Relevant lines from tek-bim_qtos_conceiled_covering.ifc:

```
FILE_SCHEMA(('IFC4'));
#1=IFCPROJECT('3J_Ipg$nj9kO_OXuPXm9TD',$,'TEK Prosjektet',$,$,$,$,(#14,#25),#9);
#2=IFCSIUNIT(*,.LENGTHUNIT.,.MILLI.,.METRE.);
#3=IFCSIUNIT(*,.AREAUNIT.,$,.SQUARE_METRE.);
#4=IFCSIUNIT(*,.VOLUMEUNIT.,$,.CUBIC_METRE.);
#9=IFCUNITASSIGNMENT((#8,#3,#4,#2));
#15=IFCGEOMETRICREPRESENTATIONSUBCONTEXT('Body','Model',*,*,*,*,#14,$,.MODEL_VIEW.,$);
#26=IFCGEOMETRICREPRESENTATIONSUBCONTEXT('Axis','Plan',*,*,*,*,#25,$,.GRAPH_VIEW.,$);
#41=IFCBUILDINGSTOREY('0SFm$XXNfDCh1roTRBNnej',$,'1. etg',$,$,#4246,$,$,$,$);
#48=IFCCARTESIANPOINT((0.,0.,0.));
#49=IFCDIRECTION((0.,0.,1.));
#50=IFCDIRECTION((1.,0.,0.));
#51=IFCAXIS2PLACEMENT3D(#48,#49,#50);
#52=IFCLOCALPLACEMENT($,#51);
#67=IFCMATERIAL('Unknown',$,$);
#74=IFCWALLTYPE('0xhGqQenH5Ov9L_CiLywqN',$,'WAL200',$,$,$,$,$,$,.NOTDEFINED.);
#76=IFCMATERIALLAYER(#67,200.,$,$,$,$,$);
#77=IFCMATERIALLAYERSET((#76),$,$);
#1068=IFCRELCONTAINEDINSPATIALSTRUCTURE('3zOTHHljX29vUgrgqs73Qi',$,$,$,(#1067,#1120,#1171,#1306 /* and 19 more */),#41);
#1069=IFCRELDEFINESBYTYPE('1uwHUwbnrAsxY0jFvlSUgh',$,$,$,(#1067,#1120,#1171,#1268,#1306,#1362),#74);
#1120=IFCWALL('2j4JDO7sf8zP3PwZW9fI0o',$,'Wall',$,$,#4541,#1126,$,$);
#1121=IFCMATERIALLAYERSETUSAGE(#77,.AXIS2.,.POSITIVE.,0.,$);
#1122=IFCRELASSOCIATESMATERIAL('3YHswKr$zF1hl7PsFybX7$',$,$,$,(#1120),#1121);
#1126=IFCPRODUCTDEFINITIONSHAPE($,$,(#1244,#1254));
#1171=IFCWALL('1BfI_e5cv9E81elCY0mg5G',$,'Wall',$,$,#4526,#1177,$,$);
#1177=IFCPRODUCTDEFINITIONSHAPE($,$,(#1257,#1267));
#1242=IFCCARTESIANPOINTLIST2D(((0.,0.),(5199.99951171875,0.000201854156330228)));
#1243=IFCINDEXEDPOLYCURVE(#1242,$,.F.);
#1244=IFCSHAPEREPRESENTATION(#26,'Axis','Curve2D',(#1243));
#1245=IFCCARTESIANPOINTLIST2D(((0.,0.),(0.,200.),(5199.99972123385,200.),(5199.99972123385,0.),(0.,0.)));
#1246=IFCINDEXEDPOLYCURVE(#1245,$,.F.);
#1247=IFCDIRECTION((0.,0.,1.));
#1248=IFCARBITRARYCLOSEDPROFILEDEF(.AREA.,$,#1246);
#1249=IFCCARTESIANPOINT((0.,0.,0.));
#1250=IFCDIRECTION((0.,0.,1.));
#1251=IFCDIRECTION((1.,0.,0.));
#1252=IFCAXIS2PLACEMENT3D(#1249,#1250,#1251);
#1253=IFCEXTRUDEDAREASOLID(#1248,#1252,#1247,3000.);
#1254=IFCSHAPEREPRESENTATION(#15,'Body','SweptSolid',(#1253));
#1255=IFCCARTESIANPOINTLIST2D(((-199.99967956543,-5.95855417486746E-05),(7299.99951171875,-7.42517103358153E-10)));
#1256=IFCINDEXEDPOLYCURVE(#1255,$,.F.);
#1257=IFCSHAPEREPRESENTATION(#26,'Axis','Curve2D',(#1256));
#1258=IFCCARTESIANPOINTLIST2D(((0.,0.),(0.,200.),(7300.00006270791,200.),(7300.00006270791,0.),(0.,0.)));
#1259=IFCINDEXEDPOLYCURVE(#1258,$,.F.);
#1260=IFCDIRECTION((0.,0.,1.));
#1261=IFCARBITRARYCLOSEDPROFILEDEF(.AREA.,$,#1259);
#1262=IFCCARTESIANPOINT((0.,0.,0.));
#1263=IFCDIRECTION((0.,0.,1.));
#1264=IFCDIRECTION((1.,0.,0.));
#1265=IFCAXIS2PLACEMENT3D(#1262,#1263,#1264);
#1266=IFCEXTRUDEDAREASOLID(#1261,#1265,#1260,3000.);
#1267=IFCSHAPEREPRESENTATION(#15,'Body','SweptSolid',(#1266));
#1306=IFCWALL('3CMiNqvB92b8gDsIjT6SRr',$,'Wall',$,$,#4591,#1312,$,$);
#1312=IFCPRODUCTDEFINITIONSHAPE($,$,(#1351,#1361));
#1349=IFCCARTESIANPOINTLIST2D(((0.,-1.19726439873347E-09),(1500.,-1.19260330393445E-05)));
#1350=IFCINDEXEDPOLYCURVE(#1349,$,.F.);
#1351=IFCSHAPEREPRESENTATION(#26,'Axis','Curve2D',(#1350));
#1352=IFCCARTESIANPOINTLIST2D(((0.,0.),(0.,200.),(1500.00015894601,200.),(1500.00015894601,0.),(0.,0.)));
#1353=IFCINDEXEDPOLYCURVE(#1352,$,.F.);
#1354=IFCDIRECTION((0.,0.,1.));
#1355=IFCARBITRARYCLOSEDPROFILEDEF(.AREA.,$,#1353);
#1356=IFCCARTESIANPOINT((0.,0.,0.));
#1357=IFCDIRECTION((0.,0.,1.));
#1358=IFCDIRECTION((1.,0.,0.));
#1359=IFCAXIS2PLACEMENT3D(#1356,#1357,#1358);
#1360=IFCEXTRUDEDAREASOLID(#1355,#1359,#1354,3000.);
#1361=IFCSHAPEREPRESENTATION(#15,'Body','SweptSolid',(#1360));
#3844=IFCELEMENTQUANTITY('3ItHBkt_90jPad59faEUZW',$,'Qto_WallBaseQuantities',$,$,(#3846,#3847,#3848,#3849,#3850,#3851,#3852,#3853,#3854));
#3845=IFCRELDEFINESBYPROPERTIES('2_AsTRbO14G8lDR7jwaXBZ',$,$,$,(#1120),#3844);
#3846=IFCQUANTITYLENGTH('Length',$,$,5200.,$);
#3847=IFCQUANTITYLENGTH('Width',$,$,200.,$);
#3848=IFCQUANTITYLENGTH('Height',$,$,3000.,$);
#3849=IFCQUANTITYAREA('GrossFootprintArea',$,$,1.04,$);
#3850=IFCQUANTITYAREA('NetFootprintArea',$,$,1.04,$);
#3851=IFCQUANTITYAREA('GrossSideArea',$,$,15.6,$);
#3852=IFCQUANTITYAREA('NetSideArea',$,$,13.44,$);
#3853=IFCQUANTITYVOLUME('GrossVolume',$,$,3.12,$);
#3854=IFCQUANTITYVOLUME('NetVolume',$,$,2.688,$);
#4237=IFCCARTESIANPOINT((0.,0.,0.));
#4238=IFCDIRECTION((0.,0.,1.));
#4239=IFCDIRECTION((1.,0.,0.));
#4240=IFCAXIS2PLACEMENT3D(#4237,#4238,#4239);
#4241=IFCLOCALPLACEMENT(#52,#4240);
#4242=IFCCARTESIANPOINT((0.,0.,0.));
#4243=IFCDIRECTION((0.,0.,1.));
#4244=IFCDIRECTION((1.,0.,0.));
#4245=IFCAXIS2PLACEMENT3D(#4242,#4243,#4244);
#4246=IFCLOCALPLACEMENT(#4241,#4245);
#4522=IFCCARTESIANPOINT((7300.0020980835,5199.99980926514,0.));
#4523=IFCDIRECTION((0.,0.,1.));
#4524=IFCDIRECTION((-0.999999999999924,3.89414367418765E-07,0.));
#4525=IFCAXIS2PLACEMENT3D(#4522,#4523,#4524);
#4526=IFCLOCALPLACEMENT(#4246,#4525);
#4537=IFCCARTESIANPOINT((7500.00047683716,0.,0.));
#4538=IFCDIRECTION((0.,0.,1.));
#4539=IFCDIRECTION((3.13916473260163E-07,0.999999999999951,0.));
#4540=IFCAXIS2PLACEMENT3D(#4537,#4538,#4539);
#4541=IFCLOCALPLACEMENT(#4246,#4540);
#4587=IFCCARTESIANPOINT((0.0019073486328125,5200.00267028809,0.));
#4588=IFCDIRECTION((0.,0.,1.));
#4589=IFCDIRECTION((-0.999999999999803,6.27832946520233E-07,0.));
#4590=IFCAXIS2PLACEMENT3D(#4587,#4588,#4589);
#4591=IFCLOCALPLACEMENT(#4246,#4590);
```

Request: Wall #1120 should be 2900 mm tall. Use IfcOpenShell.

```python
import ifcopenshell
import ifcopenshell.api.pset
import ifcopenshell.geom
import ifcopenshell.util.element
import ifcopenshell.util.representation
import ifcopenshell.util.shape
import ifcopenshell.util.unit

model = ifcopenshell.open("tek-bim_qtos_conceiled_covering.ifc")
unit_scale = ifcopenshell.util.unit.calculate_unit_scale(model)
area_scale = ifcopenshell.util.unit.calculate_unit_scale(model, "AREAUNIT")
volume_scale = ifcopenshell.util.unit.calculate_unit_scale(model, "VOLUMEUNIT")
settings = ifcopenshell.geom.settings()


def volume(element):
    """Net volume in cubic metres, openings subtracted."""
    shape = ifcopenshell.geom.create_shape(settings, element)
    return ifcopenshell.util.shape.get_volume(shape.geometry)


wall = model.by_guid("2j4JDO7sf8zP3PwZW9fI0o")
before = volume(wall)

body = ifcopenshell.util.representation.get_representation(wall, "Model", "Body")
solid = body.Items[0]
old_height = solid.Depth
solid.Depth = 2900.0
after = volume(wall)
thickness = 0.2  # wall thickness in metres

# Update the stored height, areas and volumes.
qto = model.by_id(ifcopenshell.util.element.get_pset(wall, "Qto_WallBaseQuantities", should_inherit=False)["id"])
ifcopenshell.api.pset.edit_qto(model, qto=qto, properties={
    "Height": solid.Depth,
    "GrossSideArea": ifcopenshell.util.element.get_pset(wall, "Qto_WallBaseQuantities", "GrossSideArea") * solid.Depth / old_height,
    "NetSideArea": after / thickness / area_scale,
    "GrossVolume": ifcopenshell.util.element.get_pset(wall, "Qto_WallBaseQuantities", "GrossVolume") * solid.Depth / old_height,
    "NetVolume": after / volume_scale,
})

print(f"height {old_height:g} -> {solid.Depth:g}, volume {before:.3f} -> {after:.3f} m3")

model.write("tek-bim_qtos_conceiled_covering_v2.ifc")
```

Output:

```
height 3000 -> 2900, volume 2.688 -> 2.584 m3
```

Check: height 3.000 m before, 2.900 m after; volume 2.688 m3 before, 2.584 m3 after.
